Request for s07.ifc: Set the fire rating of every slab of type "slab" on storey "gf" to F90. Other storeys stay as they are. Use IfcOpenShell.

First a look at what the model holds.

```python
import ifcopenshell
import ifcopenshell.util.element

model = ifcopenshell.open("s07.ifc")
print(model.schema)
storey = next(s for s in model.by_type("IfcBuildingStorey") if s.Name == "gf")
slabs = [e for e in ifcopenshell.util.element.get_decomposition(storey) if e.is_a("IfcSlab")]
seen = {}
for e in slabs:
    element_type = ifcopenshell.util.element.get_type(e)
    key = (element_type.Name if element_type != e and element_type else None, ifcopenshell.util.element.get_pset(e, "Pset_SlabCommon", "FireRating"))
    seen[key] = seen.get(key, 0) + 1
for (name, value), count in sorted(seen.items(), key=str):
    print(count, "x", name, "|", value)
```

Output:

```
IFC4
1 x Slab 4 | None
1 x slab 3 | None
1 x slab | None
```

```python
import ifcopenshell
import ifcopenshell.api.pset
import ifcopenshell.util.element

model = ifcopenshell.open("s07.ifc")

storey = next(s for s in model.by_type("IfcBuildingStorey") if s.Name == "gf")
slabs = [e for e in ifcopenshell.util.element.get_decomposition(storey) if e.is_a("IfcSlab")]

count = 0
for e in slabs:
    element_type = ifcopenshell.util.element.get_type(e)
    if element_type in (None, e) or element_type.Name != "slab":
        continue
    # add_pset returns the element's existing set when there is one.
    pset = ifcopenshell.api.pset.add_pset(model, product=e, name="Pset_SlabCommon")
    ifcopenshell.api.pset.edit_pset(model, pset=pset, properties={"FireRating": "F90"})
    count += 1

print(count, "slabs updated")

model.write("s07_rev.ifc")
```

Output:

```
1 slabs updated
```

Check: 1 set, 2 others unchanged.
